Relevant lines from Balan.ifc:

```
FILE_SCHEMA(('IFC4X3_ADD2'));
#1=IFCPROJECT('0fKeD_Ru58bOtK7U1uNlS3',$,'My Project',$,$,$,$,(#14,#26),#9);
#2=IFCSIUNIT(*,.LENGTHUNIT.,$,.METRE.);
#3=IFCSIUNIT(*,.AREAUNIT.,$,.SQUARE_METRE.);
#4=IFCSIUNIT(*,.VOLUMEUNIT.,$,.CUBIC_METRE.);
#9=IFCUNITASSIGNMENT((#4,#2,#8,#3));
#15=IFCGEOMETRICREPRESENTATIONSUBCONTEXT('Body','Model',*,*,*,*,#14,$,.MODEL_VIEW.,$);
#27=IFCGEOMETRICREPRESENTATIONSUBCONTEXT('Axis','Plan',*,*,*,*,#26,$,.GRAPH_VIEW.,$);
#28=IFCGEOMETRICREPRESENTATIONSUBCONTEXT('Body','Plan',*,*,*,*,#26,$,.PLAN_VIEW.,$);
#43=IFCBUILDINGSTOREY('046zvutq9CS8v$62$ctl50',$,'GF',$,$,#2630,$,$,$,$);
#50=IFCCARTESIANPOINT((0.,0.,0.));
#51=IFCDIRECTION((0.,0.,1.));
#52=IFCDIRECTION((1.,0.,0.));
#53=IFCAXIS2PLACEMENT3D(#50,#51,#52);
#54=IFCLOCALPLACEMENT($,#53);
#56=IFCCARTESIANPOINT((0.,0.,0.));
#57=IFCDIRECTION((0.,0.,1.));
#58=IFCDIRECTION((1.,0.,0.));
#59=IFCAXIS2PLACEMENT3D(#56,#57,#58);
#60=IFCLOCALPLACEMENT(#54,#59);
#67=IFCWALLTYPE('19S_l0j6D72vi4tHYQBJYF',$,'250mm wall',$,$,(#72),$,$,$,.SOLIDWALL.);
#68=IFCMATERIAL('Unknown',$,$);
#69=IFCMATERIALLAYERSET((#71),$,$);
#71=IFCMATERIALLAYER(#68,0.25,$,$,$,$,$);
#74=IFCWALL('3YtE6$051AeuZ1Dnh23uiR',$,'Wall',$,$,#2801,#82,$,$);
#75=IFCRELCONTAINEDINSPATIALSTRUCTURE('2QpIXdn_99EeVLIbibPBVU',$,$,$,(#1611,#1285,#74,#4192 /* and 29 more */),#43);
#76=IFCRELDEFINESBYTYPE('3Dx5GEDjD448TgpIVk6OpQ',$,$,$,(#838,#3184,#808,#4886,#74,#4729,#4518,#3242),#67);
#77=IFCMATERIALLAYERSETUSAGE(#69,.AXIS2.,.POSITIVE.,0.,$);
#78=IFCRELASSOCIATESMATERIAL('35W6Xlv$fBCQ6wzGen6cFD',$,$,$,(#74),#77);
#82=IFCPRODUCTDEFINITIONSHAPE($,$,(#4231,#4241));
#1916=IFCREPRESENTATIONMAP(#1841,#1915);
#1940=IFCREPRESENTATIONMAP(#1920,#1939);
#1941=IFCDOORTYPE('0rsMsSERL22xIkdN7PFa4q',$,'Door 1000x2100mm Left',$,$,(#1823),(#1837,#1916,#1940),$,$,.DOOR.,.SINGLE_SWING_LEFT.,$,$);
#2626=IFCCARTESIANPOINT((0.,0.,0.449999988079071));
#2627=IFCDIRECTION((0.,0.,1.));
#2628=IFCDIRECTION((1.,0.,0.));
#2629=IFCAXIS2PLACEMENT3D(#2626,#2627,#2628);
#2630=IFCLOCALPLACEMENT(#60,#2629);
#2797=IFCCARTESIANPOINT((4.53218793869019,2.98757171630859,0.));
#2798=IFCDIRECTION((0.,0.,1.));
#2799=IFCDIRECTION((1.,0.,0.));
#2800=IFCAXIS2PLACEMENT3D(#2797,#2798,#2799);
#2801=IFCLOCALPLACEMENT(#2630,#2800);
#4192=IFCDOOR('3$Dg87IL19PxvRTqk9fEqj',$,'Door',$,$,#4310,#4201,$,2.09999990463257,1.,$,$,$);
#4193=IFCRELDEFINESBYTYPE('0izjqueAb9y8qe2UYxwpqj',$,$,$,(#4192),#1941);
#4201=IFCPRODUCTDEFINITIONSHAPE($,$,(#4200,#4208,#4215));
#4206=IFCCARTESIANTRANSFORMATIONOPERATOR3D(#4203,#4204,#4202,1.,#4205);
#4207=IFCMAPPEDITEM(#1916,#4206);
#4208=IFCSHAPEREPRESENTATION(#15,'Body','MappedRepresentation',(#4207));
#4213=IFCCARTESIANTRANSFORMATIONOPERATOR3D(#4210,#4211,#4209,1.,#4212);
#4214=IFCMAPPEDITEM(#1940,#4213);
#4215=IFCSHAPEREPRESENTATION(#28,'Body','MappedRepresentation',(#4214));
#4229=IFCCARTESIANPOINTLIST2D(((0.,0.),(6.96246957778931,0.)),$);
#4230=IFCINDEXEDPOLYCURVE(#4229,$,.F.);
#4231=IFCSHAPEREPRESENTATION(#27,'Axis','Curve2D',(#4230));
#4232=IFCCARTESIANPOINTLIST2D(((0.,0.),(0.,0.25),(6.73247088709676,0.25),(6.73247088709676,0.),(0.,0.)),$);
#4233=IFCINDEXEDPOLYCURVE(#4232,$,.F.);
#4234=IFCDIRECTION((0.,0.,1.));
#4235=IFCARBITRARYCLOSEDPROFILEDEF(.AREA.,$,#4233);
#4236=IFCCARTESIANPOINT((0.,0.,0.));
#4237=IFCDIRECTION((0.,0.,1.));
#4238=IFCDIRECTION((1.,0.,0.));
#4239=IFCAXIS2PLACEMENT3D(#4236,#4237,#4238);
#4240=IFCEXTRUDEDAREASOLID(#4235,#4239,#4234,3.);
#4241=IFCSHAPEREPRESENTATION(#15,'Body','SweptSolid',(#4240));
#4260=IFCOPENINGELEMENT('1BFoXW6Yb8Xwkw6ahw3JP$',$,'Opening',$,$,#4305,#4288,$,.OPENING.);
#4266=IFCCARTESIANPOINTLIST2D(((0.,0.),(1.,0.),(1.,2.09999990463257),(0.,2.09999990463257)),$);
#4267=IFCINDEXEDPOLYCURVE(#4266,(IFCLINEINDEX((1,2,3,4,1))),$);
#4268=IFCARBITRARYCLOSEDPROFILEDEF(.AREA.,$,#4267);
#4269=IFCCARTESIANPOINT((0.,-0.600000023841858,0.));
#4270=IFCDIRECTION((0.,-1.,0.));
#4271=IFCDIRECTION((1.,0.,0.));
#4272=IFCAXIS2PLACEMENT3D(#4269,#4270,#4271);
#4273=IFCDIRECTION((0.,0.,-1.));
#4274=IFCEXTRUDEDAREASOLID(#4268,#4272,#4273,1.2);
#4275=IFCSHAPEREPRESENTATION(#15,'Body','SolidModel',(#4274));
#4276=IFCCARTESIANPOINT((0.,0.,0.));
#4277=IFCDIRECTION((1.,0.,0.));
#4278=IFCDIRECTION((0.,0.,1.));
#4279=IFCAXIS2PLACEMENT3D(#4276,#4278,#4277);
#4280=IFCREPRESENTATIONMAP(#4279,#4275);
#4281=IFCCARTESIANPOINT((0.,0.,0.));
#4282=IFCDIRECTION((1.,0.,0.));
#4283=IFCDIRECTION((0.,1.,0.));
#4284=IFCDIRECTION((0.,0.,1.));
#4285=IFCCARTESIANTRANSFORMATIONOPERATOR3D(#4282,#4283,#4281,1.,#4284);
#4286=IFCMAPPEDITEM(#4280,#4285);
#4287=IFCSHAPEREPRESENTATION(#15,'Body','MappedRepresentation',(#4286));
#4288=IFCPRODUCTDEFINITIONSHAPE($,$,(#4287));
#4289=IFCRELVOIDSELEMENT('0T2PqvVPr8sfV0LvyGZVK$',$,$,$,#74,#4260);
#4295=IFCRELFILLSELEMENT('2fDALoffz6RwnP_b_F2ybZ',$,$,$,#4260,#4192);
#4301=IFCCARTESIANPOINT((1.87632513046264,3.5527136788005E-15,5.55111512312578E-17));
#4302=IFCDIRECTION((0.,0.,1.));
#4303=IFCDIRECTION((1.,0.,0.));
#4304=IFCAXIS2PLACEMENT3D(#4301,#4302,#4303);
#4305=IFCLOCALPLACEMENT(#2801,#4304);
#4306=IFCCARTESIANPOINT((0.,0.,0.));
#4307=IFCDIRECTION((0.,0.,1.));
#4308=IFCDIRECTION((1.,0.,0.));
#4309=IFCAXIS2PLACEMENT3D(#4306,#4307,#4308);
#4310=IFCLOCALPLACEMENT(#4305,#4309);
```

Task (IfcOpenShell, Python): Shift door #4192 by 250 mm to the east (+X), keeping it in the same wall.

```python
import ifcopenshell
import ifcopenshell.api.geometry
import ifcopenshell.util.placement
import ifcopenshell.util.unit

model = ifcopenshell.open("Balan.ifc")
unit_scale = ifcopenshell.util.unit.calculate_unit_scale(model)

door = model.by_guid("3$Dg87IL19PxvRTqk9fEqj")
opening = door.FillsVoids[0].RelatingOpeningElement
wall = opening.VoidsElements[0].RelatingBuildingElement

wall_matrix = ifcopenshell.util.placement.get_local_placement(wall.ObjectPlacement)
shift = wall_matrix[:3, 0] * 0.25 / unit_scale
before = ifcopenshell.util.placement.get_local_placement(door.ObjectPlacement)[:3, 3].copy()

# The door is placed relative to its opening, so it follows when the opening moves.
matrix = ifcopenshell.util.placement.get_local_placement(opening.ObjectPlacement)
matrix[:3, 3] += shift
ifcopenshell.api.geometry.edit_object_placement(
    model, product=opening, matrix=matrix, is_si=False, should_transform_children=True
)

after = ifcopenshell.util.placement.get_local_placement(door.ObjectPlacement)[:3, 3]
print("door moved by", (after - before).round(3) + 0.0)

model.write("Balan_v2.ifc")
```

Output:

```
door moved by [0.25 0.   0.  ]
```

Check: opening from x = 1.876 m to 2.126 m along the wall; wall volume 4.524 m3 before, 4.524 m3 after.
